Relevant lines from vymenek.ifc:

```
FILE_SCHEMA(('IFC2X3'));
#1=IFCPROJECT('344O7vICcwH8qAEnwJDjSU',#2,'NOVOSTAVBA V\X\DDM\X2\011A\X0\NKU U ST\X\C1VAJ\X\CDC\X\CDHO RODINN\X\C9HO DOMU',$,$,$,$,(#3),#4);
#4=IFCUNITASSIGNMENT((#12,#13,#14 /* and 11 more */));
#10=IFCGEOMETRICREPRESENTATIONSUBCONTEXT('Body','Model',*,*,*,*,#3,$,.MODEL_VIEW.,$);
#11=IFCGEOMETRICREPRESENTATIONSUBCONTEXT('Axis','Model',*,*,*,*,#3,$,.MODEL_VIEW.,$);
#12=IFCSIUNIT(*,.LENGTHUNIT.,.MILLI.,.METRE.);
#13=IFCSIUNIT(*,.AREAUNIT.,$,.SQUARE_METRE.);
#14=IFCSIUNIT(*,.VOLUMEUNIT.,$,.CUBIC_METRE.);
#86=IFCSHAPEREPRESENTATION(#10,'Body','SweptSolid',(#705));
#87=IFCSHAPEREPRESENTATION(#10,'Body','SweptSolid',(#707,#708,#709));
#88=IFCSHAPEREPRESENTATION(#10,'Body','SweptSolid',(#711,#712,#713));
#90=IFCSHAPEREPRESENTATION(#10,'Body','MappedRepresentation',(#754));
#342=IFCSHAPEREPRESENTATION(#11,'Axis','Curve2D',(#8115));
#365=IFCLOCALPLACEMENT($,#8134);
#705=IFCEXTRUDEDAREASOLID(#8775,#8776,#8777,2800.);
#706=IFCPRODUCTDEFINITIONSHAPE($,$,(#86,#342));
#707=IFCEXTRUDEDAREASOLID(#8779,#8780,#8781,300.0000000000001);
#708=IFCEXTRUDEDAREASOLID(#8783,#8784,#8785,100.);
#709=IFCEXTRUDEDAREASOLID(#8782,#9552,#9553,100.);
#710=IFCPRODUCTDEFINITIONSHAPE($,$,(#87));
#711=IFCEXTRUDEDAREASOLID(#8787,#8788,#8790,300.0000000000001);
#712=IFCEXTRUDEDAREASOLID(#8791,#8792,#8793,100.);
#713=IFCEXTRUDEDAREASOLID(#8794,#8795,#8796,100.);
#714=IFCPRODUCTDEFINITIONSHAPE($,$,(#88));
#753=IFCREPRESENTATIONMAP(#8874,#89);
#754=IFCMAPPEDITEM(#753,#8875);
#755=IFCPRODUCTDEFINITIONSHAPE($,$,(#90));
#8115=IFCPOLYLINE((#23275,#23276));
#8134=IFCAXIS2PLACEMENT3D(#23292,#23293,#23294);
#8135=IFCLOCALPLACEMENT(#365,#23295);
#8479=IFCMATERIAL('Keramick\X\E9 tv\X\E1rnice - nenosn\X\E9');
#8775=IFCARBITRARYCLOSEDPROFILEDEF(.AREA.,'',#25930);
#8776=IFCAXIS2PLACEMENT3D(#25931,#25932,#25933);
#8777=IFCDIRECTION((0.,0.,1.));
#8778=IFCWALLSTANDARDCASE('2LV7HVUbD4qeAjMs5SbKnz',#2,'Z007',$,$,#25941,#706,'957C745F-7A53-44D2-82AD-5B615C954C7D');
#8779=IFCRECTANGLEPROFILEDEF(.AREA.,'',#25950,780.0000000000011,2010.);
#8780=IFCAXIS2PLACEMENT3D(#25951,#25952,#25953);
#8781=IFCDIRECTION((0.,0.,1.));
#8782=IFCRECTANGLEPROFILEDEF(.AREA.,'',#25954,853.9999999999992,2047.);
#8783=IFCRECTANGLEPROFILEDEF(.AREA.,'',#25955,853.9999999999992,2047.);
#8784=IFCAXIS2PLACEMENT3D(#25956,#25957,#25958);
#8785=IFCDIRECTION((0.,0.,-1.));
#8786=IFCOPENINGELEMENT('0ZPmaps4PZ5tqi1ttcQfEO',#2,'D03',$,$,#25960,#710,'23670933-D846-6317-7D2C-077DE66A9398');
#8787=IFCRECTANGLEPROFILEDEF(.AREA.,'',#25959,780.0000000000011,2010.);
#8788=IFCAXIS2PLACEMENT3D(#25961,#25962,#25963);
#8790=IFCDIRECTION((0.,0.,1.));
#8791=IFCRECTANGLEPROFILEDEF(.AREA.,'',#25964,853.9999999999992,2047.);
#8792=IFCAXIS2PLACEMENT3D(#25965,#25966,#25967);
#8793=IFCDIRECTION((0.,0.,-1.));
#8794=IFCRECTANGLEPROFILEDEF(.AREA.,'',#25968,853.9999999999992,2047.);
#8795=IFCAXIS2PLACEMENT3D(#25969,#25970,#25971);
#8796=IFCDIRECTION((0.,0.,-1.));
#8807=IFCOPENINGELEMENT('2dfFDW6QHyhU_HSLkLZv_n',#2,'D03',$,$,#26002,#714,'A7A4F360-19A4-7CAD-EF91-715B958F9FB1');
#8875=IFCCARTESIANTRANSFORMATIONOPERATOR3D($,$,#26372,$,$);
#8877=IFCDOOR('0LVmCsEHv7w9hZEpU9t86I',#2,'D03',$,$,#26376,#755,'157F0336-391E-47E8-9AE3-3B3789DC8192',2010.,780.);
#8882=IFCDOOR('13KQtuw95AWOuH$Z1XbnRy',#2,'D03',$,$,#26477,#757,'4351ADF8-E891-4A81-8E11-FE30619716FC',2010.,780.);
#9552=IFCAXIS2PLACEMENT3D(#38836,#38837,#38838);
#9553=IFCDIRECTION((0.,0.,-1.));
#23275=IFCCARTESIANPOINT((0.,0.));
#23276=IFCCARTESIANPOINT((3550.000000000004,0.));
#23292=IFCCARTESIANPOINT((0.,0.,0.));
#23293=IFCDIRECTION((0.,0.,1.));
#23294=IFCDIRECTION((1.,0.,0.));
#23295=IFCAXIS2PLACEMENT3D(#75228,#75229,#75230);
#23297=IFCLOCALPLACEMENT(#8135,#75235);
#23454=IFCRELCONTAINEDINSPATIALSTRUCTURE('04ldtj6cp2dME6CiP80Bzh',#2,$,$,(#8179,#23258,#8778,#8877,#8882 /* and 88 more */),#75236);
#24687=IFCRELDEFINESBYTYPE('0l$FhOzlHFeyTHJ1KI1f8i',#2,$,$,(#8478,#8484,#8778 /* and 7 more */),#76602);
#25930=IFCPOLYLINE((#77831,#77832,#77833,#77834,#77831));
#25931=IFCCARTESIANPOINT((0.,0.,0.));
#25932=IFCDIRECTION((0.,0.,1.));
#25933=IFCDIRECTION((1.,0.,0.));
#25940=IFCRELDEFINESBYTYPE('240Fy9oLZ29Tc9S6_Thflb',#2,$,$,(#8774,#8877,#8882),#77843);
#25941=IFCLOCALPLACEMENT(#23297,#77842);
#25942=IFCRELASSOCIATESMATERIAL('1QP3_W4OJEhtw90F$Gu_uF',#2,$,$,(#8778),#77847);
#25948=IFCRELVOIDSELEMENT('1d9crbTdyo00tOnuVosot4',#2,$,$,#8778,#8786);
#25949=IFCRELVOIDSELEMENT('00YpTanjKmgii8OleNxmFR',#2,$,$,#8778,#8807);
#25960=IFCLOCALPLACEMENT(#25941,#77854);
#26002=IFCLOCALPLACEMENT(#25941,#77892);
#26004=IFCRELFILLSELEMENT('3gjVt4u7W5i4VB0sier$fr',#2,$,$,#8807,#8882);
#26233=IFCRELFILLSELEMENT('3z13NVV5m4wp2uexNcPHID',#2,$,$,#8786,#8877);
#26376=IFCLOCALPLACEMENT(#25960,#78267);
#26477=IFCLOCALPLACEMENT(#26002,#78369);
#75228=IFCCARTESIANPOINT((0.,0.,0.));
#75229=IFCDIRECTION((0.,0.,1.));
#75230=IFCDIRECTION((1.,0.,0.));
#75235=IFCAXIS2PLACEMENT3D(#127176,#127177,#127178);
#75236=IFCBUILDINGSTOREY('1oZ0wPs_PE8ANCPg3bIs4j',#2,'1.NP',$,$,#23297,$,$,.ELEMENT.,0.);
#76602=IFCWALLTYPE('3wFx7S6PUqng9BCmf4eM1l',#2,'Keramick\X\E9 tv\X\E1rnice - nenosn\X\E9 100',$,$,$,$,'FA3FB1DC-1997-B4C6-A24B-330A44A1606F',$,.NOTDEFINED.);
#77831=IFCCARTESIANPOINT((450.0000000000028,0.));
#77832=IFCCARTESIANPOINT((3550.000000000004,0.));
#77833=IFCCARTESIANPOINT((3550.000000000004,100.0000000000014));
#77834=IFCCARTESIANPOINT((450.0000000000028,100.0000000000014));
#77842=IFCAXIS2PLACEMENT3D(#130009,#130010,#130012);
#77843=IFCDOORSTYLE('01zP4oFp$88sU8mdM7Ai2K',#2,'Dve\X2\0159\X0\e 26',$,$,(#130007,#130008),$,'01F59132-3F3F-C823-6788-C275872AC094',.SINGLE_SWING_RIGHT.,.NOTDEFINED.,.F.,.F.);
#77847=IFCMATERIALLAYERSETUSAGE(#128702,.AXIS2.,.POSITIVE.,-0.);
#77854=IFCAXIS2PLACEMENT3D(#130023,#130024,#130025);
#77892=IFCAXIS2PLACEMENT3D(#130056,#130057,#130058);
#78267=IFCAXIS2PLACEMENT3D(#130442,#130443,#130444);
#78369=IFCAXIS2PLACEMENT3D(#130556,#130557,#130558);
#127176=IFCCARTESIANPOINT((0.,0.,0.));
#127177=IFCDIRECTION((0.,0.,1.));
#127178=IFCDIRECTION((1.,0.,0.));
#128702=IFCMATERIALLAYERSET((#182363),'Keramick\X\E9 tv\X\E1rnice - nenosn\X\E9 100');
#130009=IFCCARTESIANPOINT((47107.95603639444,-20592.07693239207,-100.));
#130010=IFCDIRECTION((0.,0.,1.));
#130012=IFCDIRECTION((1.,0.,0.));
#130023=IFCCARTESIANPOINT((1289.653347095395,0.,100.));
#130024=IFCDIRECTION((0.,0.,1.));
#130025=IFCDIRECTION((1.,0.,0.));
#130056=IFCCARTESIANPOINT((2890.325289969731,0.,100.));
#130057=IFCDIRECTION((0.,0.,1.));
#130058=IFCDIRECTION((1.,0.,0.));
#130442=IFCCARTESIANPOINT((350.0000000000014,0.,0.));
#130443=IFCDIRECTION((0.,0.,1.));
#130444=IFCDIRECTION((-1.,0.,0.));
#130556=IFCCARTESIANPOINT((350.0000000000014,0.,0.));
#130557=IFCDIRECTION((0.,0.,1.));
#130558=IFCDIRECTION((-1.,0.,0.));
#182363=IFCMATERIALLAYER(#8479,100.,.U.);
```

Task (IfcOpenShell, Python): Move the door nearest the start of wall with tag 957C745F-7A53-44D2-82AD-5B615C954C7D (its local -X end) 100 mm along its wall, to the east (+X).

```python
import ifcopenshell
import ifcopenshell.api.geometry
import ifcopenshell.util.placement
import ifcopenshell.util.unit

model = ifcopenshell.open("vymenek.ifc")
unit_scale = ifcopenshell.util.unit.calculate_unit_scale(model)

door = model.by_guid("0LVmCsEHv7w9hZEpU9t86I")
opening = door.FillsVoids[0].RelatingOpeningElement
wall = opening.VoidsElements[0].RelatingBuildingElement

wall_matrix = ifcopenshell.util.placement.get_local_placement(wall.ObjectPlacement)
shift = wall_matrix[:3, 0] * 0.1 / unit_scale
before = ifcopenshell.util.placement.get_local_placement(door.ObjectPlacement)[:3, 3].copy()

# The door is placed relative to its opening, so it follows when the opening moves.
matrix = ifcopenshell.util.placement.get_local_placement(opening.ObjectPlacement)
matrix[:3, 3] += shift
ifcopenshell.api.geometry.edit_object_placement(
    model, product=opening, matrix=matrix, is_si=False, should_transform_children=True
)

after = ifcopenshell.util.placement.get_local_placement(door.ObjectPlacement)[:3, 3]
print("door moved by", (after - before).round(3) + 0.0)

model.write("vymenek_updated.ifc")
```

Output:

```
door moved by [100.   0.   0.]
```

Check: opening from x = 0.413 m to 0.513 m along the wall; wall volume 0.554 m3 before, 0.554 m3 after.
